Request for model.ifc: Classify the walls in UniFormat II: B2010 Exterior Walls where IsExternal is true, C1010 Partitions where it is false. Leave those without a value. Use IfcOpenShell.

First a look at what the model holds.

```python
import ifcopenshell
import ifcopenshell.util.element

model = ifcopenshell.open("model.ifc")
print(model.schema)
print("classifications:", [c.Name for c in model.by_type("IfcClassification")])
values = [ifcopenshell.util.element.get_pset(e, "Pset_WallCommon", "IsExternal") for e in model.by_type("IfcWall")]
for value in (True, False, None):
    print("IsExternal", value, values.count(value))
```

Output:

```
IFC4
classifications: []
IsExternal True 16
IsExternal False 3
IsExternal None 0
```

```python
import ifcopenshell
import ifcopenshell.api.classification
import ifcopenshell.util.element

model = ifcopenshell.open("model.ifc")

system = ifcopenshell.api.classification.add_classification(model, classification="UniFormat II")

walls = model.by_type("IfcWall")
external = {e: ifcopenshell.util.element.get_pset(e, "Pset_WallCommon", "IsExternal") for e in walls}
for flag, code, name in ((True, "B2010", "Exterior Walls"), (False, "C1010", "Partitions")):
    products = [e for e in walls if external[e] is flag]
    ifcopenshell.api.classification.add_reference(
        model, products=products, classification=system, identification=code, name=name
    )
    print(code, len(products))

model.write("model_rev.ifc")
```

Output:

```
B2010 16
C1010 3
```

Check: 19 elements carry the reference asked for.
